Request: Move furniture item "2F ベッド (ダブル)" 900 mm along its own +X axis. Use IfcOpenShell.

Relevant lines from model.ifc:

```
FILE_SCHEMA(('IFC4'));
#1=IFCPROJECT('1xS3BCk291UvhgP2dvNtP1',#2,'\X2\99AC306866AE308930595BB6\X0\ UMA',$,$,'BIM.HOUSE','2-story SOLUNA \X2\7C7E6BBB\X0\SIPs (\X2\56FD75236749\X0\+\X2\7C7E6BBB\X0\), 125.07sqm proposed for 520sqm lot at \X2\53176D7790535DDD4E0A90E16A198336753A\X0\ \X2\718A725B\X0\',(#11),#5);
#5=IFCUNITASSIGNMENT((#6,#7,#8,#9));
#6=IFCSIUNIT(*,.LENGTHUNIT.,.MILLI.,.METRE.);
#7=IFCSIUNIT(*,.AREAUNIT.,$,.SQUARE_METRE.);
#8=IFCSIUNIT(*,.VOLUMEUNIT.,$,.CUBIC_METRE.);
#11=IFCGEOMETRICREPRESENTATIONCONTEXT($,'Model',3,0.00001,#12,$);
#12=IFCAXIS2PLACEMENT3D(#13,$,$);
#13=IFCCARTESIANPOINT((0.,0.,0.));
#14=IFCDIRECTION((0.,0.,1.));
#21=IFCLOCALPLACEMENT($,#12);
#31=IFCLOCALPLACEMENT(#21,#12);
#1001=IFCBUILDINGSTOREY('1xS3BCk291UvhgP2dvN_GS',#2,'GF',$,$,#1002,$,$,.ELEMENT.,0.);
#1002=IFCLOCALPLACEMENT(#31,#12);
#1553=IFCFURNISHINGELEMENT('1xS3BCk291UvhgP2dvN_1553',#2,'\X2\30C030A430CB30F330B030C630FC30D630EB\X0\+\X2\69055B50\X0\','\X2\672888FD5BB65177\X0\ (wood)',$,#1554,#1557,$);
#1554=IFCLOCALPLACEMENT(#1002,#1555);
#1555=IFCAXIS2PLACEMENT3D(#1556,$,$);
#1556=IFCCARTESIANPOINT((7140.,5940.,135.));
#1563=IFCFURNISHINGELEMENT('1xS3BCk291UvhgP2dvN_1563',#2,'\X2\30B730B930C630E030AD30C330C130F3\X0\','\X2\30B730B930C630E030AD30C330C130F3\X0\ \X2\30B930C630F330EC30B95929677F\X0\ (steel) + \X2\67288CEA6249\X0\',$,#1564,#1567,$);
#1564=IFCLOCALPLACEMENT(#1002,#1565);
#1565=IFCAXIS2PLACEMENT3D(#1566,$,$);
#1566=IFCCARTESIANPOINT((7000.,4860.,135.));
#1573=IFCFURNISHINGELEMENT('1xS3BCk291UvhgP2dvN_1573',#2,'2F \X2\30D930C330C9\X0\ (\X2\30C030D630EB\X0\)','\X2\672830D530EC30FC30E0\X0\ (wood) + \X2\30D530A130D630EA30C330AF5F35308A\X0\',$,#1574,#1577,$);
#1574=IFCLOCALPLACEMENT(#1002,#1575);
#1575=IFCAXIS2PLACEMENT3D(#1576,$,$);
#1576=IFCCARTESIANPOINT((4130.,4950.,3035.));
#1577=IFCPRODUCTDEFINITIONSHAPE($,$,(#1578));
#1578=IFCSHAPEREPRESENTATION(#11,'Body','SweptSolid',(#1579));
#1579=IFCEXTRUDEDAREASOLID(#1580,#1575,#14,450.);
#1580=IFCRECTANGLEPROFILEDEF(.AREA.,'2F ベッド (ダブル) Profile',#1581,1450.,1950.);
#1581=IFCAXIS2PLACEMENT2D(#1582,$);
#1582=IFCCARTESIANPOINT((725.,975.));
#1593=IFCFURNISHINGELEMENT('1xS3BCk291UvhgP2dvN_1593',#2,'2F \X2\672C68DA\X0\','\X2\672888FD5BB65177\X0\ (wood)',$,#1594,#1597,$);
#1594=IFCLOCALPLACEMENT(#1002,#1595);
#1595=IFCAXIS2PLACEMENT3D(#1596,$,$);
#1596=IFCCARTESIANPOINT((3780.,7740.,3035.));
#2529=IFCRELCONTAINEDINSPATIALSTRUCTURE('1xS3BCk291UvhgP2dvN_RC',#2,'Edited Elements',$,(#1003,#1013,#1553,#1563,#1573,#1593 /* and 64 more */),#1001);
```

```python
import ifcopenshell
import ifcopenshell.api.geometry
import ifcopenshell.util.placement
import ifcopenshell.util.unit

model = ifcopenshell.open("model.ifc")
unit_scale = ifcopenshell.util.unit.calculate_unit_scale(model)

item = model.by_guid("1xS3BCk291UvhgP2dvN_1573")
matrix = ifcopenshell.util.placement.get_local_placement(item.ObjectPlacement)
matrix[:3, 3] += matrix[:3, 0] * 0.9 / unit_scale
ifcopenshell.api.geometry.edit_object_placement(model, product=item, matrix=matrix, is_si=False)

print(ifcopenshell.util.placement.get_local_placement(item.ObjectPlacement).round(3) + 0.0)

model.write("model-out.ifc")
```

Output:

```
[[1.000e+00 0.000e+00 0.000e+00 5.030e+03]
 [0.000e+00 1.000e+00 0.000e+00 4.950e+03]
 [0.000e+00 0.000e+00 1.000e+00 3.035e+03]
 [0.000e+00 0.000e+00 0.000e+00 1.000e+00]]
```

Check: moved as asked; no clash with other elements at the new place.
